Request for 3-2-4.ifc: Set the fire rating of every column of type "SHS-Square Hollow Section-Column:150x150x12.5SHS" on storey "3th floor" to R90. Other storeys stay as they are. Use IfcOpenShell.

First a look at what the model holds.

```python
import ifcopenshell
import ifcopenshell.util.element

model = ifcopenshell.open("3-2-4.ifc")
print(model.schema)
storey = next(s for s in model.by_type("IfcBuildingStorey") if s.Name == "3th floor")
columns = [e for e in ifcopenshell.util.element.get_decomposition(storey) if e.is_a("IfcColumn")]
seen = {}
for e in columns:
    element_type = ifcopenshell.util.element.get_type(e)
    key = (element_type.Name if element_type != e and element_type else None, ifcopenshell.util.element.get_pset(e, "Pset_ColumnCommon", "FireRating"))
    seen[key] = seen.get(key, 0) + 1
for (name, value), count in sorted(seen.items(), key=str):
    print(count, "x", name, "|", value)
```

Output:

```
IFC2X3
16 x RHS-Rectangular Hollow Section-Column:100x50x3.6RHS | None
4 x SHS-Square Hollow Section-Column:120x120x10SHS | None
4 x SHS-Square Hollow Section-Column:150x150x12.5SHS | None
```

```python
import ifcopenshell
import ifcopenshell.api.pset
import ifcopenshell.util.element

model = ifcopenshell.open("3-2-4.ifc")

storey = next(s for s in model.by_type("IfcBuildingStorey") if s.Name == "3th floor")
columns = [e for e in ifcopenshell.util.element.get_decomposition(storey) if e.is_a("IfcColumn")]

count = 0
for e in columns:
    element_type = ifcopenshell.util.element.get_type(e)
    if element_type in (None, e) or element_type.Name != "SHS-Square Hollow Section-Column:150x150x12.5SHS":
        continue
    # add_pset returns the element's existing set when there is one.
    pset = ifcopenshell.api.pset.add_pset(model, product=e, name="Pset_ColumnCommon")
    ifcopenshell.api.pset.edit_pset(model, pset=pset, properties={"FireRating": "R90"})
    count += 1

print(count, "columns updated")

model.write("3-2-4_v2.ifc")
```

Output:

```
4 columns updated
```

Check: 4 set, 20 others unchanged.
